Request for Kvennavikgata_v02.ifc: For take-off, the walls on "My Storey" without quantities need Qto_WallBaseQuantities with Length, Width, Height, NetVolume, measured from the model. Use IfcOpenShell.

First a look at what the model holds.

```python
import ifcopenshell
import ifcopenshell.util.element
import ifcopenshell.util.unit

model = ifcopenshell.open("Kvennavikgata_v02.ifc")
print(model.schema)
for unit_type in ("LENGTHUNIT", "AREAUNIT", "VOLUMEUNIT"):
    print(unit_type, ifcopenshell.util.unit.calculate_unit_scale(model, unit_type))
storey = next(s for s in model.by_type("IfcBuildingStorey") if s.Name == "My Storey")
walls = [e for e in ifcopenshell.util.element.get_decomposition(storey) if e.is_a("IfcWall")]
for e in sorted(walls, key=lambda e: e.id()):
    print(e.id(), e.is_a(), e.Name, list(ifcopenshell.util.element.get_psets(e, qtos_only=True)), sep=" | ")
```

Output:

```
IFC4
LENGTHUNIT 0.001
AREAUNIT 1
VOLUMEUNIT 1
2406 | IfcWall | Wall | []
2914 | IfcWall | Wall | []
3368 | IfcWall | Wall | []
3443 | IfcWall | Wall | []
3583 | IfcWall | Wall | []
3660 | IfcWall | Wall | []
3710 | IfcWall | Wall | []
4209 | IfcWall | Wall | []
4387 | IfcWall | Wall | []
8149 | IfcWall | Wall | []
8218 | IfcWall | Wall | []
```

```python
import ifcopenshell
import ifcopenshell.api.pset
import ifcopenshell.geom
import ifcopenshell.util.element
import ifcopenshell.util.shape
import ifcopenshell.util.unit

model = ifcopenshell.open("Kvennavikgata_v02.ifc")
unit_scale = ifcopenshell.util.unit.calculate_unit_scale(model)
volume_scale = ifcopenshell.util.unit.calculate_unit_scale(model, "VOLUMEUNIT")
settings = ifcopenshell.geom.settings()

storey = next(s for s in model.by_type("IfcBuildingStorey") if s.Name == "My Storey")
walls = [e for e in ifcopenshell.util.element.get_decomposition(storey) if e.is_a("IfcWall")]

for e in sorted(walls, key=lambda e: e.id()):
    if ifcopenshell.util.element.get_psets(e, qtos_only=True, should_inherit=False):
        continue
    # Geometry comes back in metres, in the element's own axes.
    shape = ifcopenshell.geom.create_shape(settings, e)
    values = {
        "Length": ifcopenshell.util.shape.get_x(shape.geometry) / unit_scale,
        "Width": ifcopenshell.util.shape.get_y(shape.geometry) / unit_scale,
        "Height": ifcopenshell.util.shape.get_z(shape.geometry) / unit_scale,
        "NetVolume": ifcopenshell.util.shape.get_volume(shape.geometry) / volume_scale,
    }
    qto = ifcopenshell.api.pset.add_qto(model, product=e, name="Qto_WallBaseQuantities")
    ifcopenshell.api.pset.edit_qto(model, qto=qto, properties=values)
    print(e.id(), {k: round(v, 3) for k, v in values.items()})

model.write("Kvennavikgata_v02_rev.ifc")
```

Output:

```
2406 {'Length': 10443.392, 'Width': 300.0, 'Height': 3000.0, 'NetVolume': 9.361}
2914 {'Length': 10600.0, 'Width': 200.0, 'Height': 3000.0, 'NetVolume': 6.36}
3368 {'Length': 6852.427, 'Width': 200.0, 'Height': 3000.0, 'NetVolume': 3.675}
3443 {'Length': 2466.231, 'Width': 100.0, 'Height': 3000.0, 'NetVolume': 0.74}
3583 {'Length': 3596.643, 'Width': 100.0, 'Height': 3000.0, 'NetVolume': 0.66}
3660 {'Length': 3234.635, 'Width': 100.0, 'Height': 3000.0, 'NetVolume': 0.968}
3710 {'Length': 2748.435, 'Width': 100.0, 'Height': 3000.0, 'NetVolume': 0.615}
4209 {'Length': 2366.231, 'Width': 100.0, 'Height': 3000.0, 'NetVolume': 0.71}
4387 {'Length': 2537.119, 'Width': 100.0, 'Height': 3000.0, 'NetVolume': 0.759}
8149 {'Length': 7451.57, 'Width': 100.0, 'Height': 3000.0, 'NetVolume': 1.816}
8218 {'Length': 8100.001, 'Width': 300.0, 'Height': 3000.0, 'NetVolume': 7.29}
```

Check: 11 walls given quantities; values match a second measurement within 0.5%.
